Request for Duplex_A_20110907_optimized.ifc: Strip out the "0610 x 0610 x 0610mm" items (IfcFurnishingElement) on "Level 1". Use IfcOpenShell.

First a look at what the model holds.

```python
import ifcopenshell
import ifcopenshell.util.element

model = ifcopenshell.open("Duplex_A_20110907_optimized.ifc")
print(model.schema)
storey = next(s for s in model.by_type("IfcBuildingStorey") if s.Name == "Level 1")
furniture = [e for e in ifcopenshell.util.element.get_decomposition(storey) if e.is_a("IfcFurnishingElement")]
seen = {}
for e in furniture:
    element_type = ifcopenshell.util.element.get_type(e)
    name = element_type.Name if element_type not in (None, e) else None
    seen[name] = seen.get(name, 0) + 1
for name, count in sorted(seen.items(), key=str):
    print(count, "x", name)
```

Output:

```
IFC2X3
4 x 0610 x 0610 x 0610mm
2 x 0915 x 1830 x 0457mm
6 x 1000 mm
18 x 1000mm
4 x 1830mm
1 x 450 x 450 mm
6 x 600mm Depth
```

```python
import ifcopenshell
import ifcopenshell.api.root
import ifcopenshell.util.element

model = ifcopenshell.open("Duplex_A_20110907_optimized.ifc")

storey = next(s for s in model.by_type("IfcBuildingStorey") if s.Name == "Level 1")
furniture = [e for e in ifcopenshell.util.element.get_decomposition(storey) if e.is_a("IfcFurnishingElement")]
targets = [e for e in furniture if (t := ifcopenshell.util.element.get_type(e)) not in (None, e) and t.Name == "0610 x 0610 x 0610mm"]

for e in targets:
    ifcopenshell.api.root.remove_product(model, product=e)
print(len(targets), "removed")

model.write("Duplex_A_20110907_optimized-out.ifc")
```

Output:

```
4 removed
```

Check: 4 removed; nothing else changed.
